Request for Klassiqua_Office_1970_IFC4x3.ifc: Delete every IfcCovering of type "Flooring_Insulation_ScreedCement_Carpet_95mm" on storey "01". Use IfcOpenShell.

First a look at what the model holds.

```python
import ifcopenshell
import ifcopenshell.util.element

model = ifcopenshell.open("Klassiqua_Office_1970_IFC4x3.ifc")
print(model.schema)
storey = next(s for s in model.by_type("IfcBuildingStorey") if s.Name == "01")
coverings = [e for e in ifcopenshell.util.element.get_decomposition(storey) if e.is_a("IfcCovering")]
seen = {}
for e in coverings:
    element_type = ifcopenshell.util.element.get_type(e)
    name = element_type.Name if element_type not in (None, e) else None
    seen[name] = seen.get(name, 0) + 1
for name, count in sorted(seen.items(), key=str):
    print(count, "x", name)
```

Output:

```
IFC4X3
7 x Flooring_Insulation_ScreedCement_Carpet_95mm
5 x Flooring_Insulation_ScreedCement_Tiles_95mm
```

```python
import ifcopenshell
import ifcopenshell.api.root
import ifcopenshell.util.element

model = ifcopenshell.open("Klassiqua_Office_1970_IFC4x3.ifc")

storey = next(s for s in model.by_type("IfcBuildingStorey") if s.Name == "01")
coverings = [e for e in ifcopenshell.util.element.get_decomposition(storey) if e.is_a("IfcCovering")]
targets = [e for e in coverings if (t := ifcopenshell.util.element.get_type(e)) not in (None, e) and t.Name == "Flooring_Insulation_ScreedCement_Carpet_95mm"]

for e in targets:
    ifcopenshell.api.root.remove_product(model, product=e)
print(len(targets), "removed")

model.write("Klassiqua_Office_1970_IFC4x3_updated.ifc")
```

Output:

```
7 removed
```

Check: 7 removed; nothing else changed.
